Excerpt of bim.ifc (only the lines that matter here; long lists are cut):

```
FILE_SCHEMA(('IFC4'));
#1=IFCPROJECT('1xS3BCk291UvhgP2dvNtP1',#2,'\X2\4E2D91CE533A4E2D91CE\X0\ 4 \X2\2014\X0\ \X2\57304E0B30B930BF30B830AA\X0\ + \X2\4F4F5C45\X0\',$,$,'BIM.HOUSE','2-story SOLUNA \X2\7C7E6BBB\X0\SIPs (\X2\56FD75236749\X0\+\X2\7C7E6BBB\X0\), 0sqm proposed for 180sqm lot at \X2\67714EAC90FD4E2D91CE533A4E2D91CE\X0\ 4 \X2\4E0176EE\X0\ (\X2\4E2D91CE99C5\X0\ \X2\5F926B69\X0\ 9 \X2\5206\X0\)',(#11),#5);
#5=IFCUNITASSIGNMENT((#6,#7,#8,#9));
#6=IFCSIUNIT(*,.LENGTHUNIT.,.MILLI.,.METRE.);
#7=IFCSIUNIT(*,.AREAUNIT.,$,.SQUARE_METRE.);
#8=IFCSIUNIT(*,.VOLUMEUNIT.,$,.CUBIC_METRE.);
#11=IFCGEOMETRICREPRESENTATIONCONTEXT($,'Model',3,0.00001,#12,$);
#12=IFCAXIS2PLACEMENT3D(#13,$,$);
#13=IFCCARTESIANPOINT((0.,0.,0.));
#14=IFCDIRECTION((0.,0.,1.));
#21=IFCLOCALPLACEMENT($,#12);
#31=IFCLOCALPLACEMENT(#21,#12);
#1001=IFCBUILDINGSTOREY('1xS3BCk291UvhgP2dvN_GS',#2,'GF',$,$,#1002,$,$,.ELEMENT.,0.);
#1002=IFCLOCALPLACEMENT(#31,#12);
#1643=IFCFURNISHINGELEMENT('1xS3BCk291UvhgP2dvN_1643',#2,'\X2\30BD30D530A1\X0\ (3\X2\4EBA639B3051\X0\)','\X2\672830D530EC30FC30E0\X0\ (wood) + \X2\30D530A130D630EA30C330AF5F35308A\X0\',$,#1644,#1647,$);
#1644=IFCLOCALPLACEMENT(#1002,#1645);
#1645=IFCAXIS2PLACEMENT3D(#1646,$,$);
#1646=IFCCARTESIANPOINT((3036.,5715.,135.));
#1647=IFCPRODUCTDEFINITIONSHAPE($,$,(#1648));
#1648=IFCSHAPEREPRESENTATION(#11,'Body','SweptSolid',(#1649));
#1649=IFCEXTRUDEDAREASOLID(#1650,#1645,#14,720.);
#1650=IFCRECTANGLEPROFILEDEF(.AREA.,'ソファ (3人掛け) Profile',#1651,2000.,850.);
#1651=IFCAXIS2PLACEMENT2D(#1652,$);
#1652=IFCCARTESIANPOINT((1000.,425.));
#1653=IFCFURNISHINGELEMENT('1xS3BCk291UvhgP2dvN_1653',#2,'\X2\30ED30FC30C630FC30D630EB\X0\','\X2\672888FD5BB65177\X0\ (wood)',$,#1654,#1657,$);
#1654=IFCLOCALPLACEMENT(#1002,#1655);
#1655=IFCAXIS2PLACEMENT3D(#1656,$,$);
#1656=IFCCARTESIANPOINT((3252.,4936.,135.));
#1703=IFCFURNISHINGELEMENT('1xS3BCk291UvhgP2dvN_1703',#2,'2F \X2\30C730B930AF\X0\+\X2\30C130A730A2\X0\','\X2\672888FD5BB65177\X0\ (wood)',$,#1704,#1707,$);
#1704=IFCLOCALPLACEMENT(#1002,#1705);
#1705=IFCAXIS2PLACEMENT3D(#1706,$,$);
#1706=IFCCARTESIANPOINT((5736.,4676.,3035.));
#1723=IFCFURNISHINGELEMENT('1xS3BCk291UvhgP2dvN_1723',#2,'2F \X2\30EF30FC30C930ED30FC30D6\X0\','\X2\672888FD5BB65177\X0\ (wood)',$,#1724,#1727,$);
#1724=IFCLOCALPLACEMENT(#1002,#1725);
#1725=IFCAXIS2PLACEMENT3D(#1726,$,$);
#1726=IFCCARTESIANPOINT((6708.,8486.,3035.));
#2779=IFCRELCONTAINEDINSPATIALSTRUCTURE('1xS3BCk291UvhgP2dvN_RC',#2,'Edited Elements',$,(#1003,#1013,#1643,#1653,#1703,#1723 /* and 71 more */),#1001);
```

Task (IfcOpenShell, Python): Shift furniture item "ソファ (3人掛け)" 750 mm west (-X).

```python
import ifcopenshell
import ifcopenshell.api.geometry
import ifcopenshell.util.placement
import ifcopenshell.util.unit

model = ifcopenshell.open("bim.ifc")
unit_scale = ifcopenshell.util.unit.calculate_unit_scale(model)

item = model.by_guid("1xS3BCk291UvhgP2dvN_1643")
matrix = ifcopenshell.util.placement.get_local_placement(item.ObjectPlacement)
matrix[0, 3] -= 0.75 / unit_scale
ifcopenshell.api.geometry.edit_object_placement(model, product=item, matrix=matrix, is_si=False)

print(ifcopenshell.util.placement.get_local_placement(item.ObjectPlacement).round(3) + 0.0)

model.write("bim_v2.ifc")
```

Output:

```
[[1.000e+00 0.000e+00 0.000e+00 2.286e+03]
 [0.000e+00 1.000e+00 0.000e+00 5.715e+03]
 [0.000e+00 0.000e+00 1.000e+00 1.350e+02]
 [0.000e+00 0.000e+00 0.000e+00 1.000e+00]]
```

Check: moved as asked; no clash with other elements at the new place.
